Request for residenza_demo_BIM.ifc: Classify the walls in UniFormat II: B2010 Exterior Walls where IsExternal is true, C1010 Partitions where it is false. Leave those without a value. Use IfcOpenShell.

First a look at what the model holds.

```python
import ifcopenshell
import ifcopenshell.util.element

model = ifcopenshell.open("residenza_demo_BIM.ifc")
print(model.schema)
print("classifications:", [c.Name for c in model.by_type("IfcClassification")])
values = [ifcopenshell.util.element.get_pset(e, "Pset_WallCommon", "IsExternal") for e in model.by_type("IfcWall")]
for value in (True, False, None):
    print("IsExternal", value, values.count(value))
```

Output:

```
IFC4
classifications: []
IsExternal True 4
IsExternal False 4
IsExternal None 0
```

```python
import ifcopenshell
import ifcopenshell.api.classification
import ifcopenshell.util.element

model = ifcopenshell.open("residenza_demo_BIM.ifc")

system = ifcopenshell.api.classification.add_classification(model, classification="UniFormat II")

walls = model.by_type("IfcWall")
external = {e: ifcopenshell.util.element.get_pset(e, "Pset_WallCommon", "IsExternal") for e in walls}
for flag, code, name in ((True, "B2010", "Exterior Walls"), (False, "C1010", "Partitions")):
    products = [e for e in walls if external[e] is flag]
    ifcopenshell.api.classification.add_reference(
        model, products=products, classification=system, identification=code, name=name
    )
    print(code, len(products))

model.write("residenza_demo_BIM_rev.ifc")
```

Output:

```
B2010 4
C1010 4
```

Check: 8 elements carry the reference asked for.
